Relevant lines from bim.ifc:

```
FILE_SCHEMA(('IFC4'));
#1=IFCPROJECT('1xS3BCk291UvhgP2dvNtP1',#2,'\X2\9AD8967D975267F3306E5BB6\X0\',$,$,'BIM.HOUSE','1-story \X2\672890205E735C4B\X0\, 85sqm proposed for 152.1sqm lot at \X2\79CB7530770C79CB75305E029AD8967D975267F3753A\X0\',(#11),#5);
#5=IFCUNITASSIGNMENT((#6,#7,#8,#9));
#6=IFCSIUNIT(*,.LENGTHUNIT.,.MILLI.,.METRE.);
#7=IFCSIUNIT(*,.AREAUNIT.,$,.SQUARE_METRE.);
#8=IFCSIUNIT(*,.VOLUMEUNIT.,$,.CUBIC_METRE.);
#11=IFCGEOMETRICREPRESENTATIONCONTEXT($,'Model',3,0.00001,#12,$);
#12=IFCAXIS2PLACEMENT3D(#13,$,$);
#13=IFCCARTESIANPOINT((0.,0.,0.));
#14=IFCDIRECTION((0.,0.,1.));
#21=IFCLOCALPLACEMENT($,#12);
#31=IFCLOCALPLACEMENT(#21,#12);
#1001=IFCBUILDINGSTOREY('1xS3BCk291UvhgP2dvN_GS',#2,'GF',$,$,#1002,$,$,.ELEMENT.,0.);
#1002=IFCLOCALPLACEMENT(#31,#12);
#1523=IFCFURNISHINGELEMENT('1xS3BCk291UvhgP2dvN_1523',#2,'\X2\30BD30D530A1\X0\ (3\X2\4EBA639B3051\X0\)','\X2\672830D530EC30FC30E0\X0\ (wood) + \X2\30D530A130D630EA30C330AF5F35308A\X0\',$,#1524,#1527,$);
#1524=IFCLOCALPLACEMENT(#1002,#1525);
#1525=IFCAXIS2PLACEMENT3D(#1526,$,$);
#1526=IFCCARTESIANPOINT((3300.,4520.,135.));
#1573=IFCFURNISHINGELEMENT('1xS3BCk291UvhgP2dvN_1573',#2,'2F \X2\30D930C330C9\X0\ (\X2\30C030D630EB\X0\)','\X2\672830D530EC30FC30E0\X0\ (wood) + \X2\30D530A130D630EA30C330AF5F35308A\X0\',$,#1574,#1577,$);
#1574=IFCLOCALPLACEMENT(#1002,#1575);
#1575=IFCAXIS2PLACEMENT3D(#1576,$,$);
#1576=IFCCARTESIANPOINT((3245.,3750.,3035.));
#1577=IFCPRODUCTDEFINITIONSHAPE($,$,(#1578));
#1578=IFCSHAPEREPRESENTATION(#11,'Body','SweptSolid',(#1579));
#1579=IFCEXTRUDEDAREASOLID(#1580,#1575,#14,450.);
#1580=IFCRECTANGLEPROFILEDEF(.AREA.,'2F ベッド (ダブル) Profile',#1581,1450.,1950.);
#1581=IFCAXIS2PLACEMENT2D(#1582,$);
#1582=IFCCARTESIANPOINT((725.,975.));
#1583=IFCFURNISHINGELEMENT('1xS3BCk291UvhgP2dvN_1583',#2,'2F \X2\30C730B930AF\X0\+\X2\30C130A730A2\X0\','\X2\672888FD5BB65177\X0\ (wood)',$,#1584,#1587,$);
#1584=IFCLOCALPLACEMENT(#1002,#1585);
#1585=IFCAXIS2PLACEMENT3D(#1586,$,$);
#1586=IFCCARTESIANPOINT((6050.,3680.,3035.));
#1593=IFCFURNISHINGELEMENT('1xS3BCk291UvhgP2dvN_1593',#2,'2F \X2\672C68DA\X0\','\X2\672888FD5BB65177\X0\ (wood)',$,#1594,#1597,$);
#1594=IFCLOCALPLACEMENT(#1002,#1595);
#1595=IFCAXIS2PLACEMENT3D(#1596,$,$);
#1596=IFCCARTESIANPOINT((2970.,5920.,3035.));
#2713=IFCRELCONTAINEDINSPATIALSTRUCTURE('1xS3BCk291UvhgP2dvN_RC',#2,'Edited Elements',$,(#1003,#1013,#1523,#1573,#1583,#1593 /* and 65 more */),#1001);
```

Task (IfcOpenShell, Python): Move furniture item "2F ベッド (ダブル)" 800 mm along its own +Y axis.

```python
import ifcopenshell
import ifcopenshell.api.geometry
import ifcopenshell.util.placement

model = ifcopenshell.open("bim.ifc")

item = model.by_guid("1xS3BCk291UvhgP2dvN_1573")
matrix = ifcopenshell.util.placement.get_local_placement(item.ObjectPlacement)
matrix[:3, 3] += matrix[:3, 1] * 800.0
ifcopenshell.api.geometry.edit_object_placement(model, product=item, matrix=matrix, is_si=False)

print(ifcopenshell.util.placement.get_local_placement(item.ObjectPlacement).round(3) + 0.0)

model.write("bim_v2.ifc")
```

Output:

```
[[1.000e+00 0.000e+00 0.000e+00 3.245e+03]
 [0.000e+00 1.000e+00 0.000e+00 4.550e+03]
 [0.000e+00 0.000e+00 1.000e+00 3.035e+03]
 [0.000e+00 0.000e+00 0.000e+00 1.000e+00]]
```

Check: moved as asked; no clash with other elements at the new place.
